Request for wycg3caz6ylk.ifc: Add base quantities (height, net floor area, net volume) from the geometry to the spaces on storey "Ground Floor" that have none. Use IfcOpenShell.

First a look at what the model holds.

```python
import ifcopenshell
import ifcopenshell.util.element
import ifcopenshell.util.unit

model = ifcopenshell.open("wycg3caz6ylk.ifc")
print(model.schema)
for unit_type in ("LENGTHUNIT", "AREAUNIT", "VOLUMEUNIT"):
    print(unit_type, ifcopenshell.util.unit.calculate_unit_scale(model, unit_type))
storey = next(s for s in model.by_type("IfcBuildingStorey") if s.Name == "Ground Floor")
spaces = [e for e in ifcopenshell.util.element.get_decomposition(storey) if e.is_a("IfcSpace")]
for e in sorted(spaces, key=lambda e: e.id()):
    print(e.id(), e.is_a(), e.Name, list(ifcopenshell.util.element.get_psets(e, qtos_only=True)), sep=" | ")
```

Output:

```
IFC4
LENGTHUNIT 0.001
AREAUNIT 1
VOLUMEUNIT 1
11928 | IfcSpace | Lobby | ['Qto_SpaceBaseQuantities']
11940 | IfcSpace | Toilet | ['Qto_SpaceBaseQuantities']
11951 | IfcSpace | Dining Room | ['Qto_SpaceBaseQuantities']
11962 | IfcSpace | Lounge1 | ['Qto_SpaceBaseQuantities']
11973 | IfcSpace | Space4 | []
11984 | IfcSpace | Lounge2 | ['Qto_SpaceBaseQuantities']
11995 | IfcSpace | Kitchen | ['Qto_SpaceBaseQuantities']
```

```python
import ifcopenshell
import ifcopenshell.api.pset
import ifcopenshell.geom
import ifcopenshell.util.element
import ifcopenshell.util.shape
import ifcopenshell.util.unit

model = ifcopenshell.open("wycg3caz6ylk.ifc")
unit_scale = ifcopenshell.util.unit.calculate_unit_scale(model)
area_scale = ifcopenshell.util.unit.calculate_unit_scale(model, "AREAUNIT")
volume_scale = ifcopenshell.util.unit.calculate_unit_scale(model, "VOLUMEUNIT")
settings = ifcopenshell.geom.settings()

storey = next(s for s in model.by_type("IfcBuildingStorey") if s.Name == "Ground Floor")
spaces = [e for e in ifcopenshell.util.element.get_decomposition(storey) if e.is_a("IfcSpace")]

for e in sorted(spaces, key=lambda e: e.id()):
    if ifcopenshell.util.element.get_psets(e, qtos_only=True, should_inherit=False):
        continue
    # Geometry comes back in metres, in the element's own axes.
    shape = ifcopenshell.geom.create_shape(settings, e)
    values = {
        "Height": ifcopenshell.util.shape.get_z(shape.geometry) / unit_scale,
        "NetFloorArea": ifcopenshell.util.shape.get_footprint_area(shape.geometry) / area_scale,
        "NetVolume": ifcopenshell.util.shape.get_volume(shape.geometry) / volume_scale,
    }
    qto = ifcopenshell.api.pset.add_qto(model, product=e, name="Qto_SpaceBaseQuantities")
    ifcopenshell.api.pset.edit_qto(model, qto=qto, properties=values)
    print(e.id(), {k: round(v, 3) for k, v in values.items()})

model.write("wycg3caz6ylk_edited.ifc")
```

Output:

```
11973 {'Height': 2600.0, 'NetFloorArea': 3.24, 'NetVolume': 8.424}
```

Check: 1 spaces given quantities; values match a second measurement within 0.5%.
